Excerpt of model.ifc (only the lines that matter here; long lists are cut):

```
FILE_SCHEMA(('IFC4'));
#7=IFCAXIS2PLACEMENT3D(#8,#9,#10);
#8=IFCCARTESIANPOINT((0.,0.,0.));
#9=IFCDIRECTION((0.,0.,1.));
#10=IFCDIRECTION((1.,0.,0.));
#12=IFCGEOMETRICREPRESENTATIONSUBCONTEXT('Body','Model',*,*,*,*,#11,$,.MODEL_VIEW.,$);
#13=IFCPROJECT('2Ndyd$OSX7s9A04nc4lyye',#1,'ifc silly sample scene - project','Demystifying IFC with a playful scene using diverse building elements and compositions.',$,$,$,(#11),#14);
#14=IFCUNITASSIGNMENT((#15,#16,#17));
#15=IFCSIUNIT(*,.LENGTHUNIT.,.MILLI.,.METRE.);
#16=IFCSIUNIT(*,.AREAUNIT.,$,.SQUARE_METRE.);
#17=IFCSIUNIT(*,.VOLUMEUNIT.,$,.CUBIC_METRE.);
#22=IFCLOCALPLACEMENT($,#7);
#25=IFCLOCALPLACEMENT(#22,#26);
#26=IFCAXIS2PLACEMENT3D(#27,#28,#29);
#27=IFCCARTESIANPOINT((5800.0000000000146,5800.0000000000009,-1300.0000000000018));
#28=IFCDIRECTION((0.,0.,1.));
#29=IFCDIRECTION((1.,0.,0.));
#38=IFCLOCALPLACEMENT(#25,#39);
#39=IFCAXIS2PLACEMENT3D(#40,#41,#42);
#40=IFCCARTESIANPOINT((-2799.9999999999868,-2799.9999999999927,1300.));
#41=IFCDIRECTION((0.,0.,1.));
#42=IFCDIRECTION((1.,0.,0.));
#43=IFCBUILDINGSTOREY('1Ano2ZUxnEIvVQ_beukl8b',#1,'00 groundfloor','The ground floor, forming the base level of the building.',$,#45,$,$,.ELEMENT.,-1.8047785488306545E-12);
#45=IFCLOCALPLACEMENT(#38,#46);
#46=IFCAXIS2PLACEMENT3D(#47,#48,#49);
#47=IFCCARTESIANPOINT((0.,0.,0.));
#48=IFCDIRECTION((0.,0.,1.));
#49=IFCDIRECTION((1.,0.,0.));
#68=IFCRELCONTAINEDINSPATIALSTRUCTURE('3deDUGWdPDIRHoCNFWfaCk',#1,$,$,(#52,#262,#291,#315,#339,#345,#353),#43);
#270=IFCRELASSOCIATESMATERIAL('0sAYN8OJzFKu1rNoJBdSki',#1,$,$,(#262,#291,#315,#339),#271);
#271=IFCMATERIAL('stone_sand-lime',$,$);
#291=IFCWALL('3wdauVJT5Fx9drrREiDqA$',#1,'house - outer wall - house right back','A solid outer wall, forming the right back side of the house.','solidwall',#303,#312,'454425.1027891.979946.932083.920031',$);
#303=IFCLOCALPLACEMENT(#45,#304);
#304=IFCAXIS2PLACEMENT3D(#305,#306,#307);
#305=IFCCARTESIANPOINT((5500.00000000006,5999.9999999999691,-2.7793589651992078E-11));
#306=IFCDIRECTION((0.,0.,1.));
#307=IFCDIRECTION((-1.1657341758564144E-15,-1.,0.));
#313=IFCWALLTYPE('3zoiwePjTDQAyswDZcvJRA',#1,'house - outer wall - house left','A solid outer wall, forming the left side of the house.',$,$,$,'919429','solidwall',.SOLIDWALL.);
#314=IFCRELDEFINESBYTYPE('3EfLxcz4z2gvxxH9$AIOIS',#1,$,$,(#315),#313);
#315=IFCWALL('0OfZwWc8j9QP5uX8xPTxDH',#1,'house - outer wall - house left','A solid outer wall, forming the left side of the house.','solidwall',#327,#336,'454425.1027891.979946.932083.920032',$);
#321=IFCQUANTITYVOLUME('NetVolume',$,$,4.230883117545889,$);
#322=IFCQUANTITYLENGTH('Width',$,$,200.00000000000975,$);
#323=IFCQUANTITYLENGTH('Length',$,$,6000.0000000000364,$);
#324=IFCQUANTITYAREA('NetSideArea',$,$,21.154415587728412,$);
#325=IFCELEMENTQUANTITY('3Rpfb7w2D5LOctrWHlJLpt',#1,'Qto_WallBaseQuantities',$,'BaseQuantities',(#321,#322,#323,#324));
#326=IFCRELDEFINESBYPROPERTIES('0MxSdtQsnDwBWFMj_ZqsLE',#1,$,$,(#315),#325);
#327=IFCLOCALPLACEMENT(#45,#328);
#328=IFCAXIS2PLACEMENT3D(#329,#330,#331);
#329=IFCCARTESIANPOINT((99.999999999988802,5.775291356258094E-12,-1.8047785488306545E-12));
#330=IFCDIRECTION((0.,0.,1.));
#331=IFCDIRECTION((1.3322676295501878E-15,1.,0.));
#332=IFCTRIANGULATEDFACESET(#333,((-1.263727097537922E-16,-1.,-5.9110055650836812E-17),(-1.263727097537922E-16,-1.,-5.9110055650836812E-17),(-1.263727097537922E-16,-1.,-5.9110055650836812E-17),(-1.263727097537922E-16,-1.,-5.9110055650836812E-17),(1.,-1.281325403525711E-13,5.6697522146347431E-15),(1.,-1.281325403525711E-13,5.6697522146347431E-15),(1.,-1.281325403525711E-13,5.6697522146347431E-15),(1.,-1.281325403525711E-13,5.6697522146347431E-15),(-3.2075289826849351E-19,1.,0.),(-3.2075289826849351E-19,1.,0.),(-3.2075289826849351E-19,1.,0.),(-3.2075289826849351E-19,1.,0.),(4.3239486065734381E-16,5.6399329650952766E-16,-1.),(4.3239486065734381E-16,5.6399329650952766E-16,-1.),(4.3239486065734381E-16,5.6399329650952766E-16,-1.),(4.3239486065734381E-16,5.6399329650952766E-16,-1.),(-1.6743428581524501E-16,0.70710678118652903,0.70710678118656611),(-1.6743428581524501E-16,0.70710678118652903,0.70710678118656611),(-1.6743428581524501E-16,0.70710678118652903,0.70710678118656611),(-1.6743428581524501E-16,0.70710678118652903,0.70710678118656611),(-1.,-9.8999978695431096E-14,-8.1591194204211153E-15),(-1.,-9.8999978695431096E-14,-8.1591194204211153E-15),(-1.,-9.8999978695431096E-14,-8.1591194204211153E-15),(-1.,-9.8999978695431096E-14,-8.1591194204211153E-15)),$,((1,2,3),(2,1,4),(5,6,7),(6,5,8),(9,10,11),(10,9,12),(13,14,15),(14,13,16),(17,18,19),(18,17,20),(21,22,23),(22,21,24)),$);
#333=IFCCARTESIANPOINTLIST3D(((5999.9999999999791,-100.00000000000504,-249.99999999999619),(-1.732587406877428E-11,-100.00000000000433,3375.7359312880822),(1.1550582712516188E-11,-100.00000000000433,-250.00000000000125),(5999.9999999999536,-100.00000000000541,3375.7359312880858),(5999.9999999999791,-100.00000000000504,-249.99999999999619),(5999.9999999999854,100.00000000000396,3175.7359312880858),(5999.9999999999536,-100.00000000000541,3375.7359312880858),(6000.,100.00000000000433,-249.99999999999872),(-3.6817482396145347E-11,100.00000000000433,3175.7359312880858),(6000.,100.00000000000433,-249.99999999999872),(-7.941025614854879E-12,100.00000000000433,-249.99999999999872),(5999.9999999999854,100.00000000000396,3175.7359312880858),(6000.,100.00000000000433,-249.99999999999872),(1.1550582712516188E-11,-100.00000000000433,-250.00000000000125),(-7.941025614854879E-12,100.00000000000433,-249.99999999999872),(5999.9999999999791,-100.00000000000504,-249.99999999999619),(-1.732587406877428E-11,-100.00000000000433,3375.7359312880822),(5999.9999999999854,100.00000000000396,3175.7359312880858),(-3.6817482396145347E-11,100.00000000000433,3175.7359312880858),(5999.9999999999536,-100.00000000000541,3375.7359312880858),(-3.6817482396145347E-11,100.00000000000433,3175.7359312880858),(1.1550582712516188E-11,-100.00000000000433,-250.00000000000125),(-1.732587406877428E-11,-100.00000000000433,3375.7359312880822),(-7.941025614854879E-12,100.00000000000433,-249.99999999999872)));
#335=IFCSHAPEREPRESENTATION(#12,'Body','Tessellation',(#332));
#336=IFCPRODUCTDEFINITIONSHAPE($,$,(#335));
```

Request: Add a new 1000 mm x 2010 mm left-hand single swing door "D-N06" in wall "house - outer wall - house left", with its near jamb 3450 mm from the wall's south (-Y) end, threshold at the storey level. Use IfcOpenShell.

```python
import numpy as np
import ifcopenshell
import ifcopenshell.api.feature
import ifcopenshell.api.geometry
import ifcopenshell.api.pset
import ifcopenshell.api.root
import ifcopenshell.api.spatial
import ifcopenshell.geom
import ifcopenshell.util.element
import ifcopenshell.util.placement
import ifcopenshell.util.representation
import ifcopenshell.util.shape
import ifcopenshell.util.unit

model = ifcopenshell.open("model.ifc")
unit_scale = ifcopenshell.util.unit.calculate_unit_scale(model)
area_scale = ifcopenshell.util.unit.calculate_unit_scale(model, "AREAUNIT")
volume_scale = ifcopenshell.util.unit.calculate_unit_scale(model, "VOLUMEUNIT")
settings = ifcopenshell.geom.settings()


def volume(element):
    """Net volume in cubic metres, openings subtracted."""
    shape = ifcopenshell.geom.create_shape(settings, element)
    return ifcopenshell.util.shape.get_volume(shape.geometry)


wall = model.by_guid("0OfZwWc8j9QP5uX8xPTxDH")
storey = ifcopenshell.util.element.get_container(wall, ifc_class="IfcBuildingStorey")
context = ifcopenshell.util.representation.get_context(model, "Model", "Body", "MODEL_VIEW")
before = volume(wall)

width, height, from_end, sill = 1, 2.01, 3.45, 0.0  # metres

# The wall runs along its own X axis, and the end named is its -X end.
wall_shape = ifcopenshell.geom.create_shape(settings, wall)
x, y, z = ifcopenshell.util.shape.get_vertices(wall_shape.geometry).T
start = x.min() + from_end
face, thickness = float(y.min()), float(y.max() - y.min())
wall_matrix = ifcopenshell.util.placement.get_local_placement(wall.ObjectPlacement)
level = ifcopenshell.util.placement.get_local_placement(storey.ObjectPlacement)[2, 3]


def in_wall(x, y):
    """Placement at x, y metres in the wall's axes, at sill height."""
    matrix = wall_matrix.copy()
    matrix[:, 3] = wall_matrix @ np.array([x / unit_scale, y / unit_scale, 0.0, 1.0])
    matrix[2, 3] = level + sill / unit_scale
    return matrix


# Opening: a box that overshoots both wall faces by 50 mm.
opening = ifcopenshell.api.root.create_entity(model, ifc_class="IfcOpeningElement", predefined_type="OPENING")
box = ifcopenshell.api.geometry.add_wall_representation(
    model, context=context, length=width, height=height, thickness=thickness + 0.1
)
ifcopenshell.api.geometry.assign_representation(model, product=opening, representation=box)
ifcopenshell.api.geometry.edit_object_placement(model, product=opening, matrix=in_wall(start, face - 0.05), is_si=False)
ifcopenshell.api.feature.add_feature(model, feature=opening, element=wall)

door = ifcopenshell.api.root.create_entity(model, ifc_class="IfcDoor", name="D-N06", predefined_type="DOOR")
door.OverallWidth, door.OverallHeight = width / unit_scale, height / unit_scale
door.OperationType = "SINGLE_SWING_LEFT"
body = ifcopenshell.api.geometry.add_door_representation(
    model,
    context=context,
    overall_width=door.OverallWidth,
    overall_height=door.OverallHeight,
    operation_type="SINGLE_SWING_LEFT",
    lining_properties={"LiningDepth": thickness / unit_scale, "ThresholdDepth": thickness / unit_scale},
)
ifcopenshell.api.geometry.assign_representation(model, product=door, representation=body)
ifcopenshell.api.spatial.assign_container(model, products=[door], relating_structure=storey)
ifcopenshell.api.feature.add_filling(model, opening=opening, element=door)

# The lining spans the wall, so the door starts at the wall face.
ifcopenshell.api.geometry.edit_object_placement(model, product=door, matrix=in_wall(start, face), is_si=False)

after = volume(wall)

# Update the wall's stored quantities.
qto = model.by_id(ifcopenshell.util.element.get_pset(wall, "Qto_WallBaseQuantities", should_inherit=False)["id"])
ifcopenshell.api.pset.edit_qto(model, qto=qto, properties={
    "NetVolume": after / volume_scale,
    "NetSideArea": after / thickness / area_scale,
})

print(f"wall volume {before:.3f} -> {after:.3f} m3")

model.write("model_edited.ifc")
```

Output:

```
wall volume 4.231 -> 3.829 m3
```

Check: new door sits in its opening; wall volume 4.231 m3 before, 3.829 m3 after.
